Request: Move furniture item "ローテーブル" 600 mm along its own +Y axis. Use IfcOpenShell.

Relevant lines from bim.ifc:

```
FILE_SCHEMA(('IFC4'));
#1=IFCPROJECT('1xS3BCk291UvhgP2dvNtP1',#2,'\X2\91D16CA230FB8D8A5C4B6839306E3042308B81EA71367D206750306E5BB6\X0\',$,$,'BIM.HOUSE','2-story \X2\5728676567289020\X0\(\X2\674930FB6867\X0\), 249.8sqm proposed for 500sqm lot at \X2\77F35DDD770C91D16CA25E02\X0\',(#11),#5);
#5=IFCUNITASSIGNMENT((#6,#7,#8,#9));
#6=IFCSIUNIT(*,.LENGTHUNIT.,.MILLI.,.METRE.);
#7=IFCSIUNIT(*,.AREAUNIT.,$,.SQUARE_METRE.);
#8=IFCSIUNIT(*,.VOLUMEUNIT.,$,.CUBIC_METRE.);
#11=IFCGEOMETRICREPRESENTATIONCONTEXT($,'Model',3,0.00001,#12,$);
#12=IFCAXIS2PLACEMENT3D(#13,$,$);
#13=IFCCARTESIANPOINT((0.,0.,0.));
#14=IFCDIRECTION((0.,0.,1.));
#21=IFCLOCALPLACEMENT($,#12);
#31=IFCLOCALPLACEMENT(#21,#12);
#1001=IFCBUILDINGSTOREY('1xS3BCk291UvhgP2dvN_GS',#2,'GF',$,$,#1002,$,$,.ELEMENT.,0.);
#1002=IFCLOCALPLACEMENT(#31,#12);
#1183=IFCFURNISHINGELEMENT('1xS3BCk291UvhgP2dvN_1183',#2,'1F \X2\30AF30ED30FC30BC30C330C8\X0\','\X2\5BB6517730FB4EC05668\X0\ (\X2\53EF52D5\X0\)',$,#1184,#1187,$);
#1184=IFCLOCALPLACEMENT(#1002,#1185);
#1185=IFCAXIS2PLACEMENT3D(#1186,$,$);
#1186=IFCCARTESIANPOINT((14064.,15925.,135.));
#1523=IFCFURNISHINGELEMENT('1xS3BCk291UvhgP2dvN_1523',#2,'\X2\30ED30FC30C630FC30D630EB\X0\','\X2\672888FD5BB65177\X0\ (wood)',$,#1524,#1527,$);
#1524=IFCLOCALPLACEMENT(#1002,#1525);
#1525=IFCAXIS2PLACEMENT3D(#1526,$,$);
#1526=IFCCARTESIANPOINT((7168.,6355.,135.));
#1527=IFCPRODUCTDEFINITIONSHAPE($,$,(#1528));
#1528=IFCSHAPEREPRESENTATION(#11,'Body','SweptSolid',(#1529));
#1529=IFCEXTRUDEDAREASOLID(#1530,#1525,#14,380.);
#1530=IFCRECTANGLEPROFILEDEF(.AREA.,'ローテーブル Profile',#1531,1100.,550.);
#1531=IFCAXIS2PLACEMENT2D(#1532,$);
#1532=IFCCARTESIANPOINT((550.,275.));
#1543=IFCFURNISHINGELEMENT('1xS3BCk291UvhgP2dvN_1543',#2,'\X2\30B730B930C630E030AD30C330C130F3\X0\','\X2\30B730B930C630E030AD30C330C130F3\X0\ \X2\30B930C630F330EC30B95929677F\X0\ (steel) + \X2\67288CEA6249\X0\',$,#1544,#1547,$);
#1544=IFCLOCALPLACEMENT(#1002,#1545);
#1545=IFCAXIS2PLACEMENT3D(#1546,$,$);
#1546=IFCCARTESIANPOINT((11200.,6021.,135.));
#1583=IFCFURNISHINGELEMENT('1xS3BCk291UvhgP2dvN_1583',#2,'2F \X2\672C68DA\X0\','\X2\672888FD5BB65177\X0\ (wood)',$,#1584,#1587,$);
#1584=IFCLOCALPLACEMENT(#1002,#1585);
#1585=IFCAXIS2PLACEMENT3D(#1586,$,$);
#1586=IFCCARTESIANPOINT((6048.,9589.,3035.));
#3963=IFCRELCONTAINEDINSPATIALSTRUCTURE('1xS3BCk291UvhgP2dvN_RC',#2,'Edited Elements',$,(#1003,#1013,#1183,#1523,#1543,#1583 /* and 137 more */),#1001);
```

```python
import ifcopenshell
import ifcopenshell.api.geometry
import ifcopenshell.util.placement
import ifcopenshell.util.unit

model = ifcopenshell.open("bim.ifc")
unit_scale = ifcopenshell.util.unit.calculate_unit_scale(model)

item = model.by_id(1523)
matrix = ifcopenshell.util.placement.get_local_placement(item.ObjectPlacement)
matrix[:3, 3] += matrix[:3, 1] * 0.6 / unit_scale
ifcopenshell.api.geometry.edit_object_placement(model, product=item, matrix=matrix, is_si=False)

print(ifcopenshell.util.placement.get_local_placement(item.ObjectPlacement).round(3) + 0.0)

model.write("bim-out.ifc")
```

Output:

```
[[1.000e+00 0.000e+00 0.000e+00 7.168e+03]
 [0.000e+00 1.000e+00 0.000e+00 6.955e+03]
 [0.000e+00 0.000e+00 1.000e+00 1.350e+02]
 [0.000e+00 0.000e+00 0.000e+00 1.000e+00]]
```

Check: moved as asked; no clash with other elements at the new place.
